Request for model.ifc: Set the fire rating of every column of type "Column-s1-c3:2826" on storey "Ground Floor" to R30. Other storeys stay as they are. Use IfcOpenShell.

First a look at what the model holds.

```python
import ifcopenshell
import ifcopenshell.util.element

model = ifcopenshell.open("model.ifc")
print(model.schema)
storey = next(s for s in model.by_type("IfcBuildingStorey") if s.Name == "Ground Floor")
columns = [e for e in ifcopenshell.util.element.get_decomposition(storey) if e.is_a("IfcColumn")]
seen = {}
for e in columns:
    element_type = ifcopenshell.util.element.get_type(e)
    key = (element_type.Name if element_type != e and element_type else None, ifcopenshell.util.element.get_pset(e, "Pset_ColumnCommon", "FireRating"))
    seen[key] = seen.get(key, 0) + 1
for (name, value), count in sorted(seen.items(), key=str):
    print(count, "x", name, "|", value)
```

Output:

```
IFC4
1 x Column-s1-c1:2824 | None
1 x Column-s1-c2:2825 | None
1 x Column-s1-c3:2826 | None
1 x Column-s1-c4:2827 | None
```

```python
import ifcopenshell
import ifcopenshell.api.pset
import ifcopenshell.util.element

model = ifcopenshell.open("model.ifc")

storey = next(s for s in model.by_type("IfcBuildingStorey") if s.Name == "Ground Floor")
columns = [e for e in ifcopenshell.util.element.get_decomposition(storey) if e.is_a("IfcColumn")]

count = 0
for e in columns:
    element_type = ifcopenshell.util.element.get_type(e)
    if element_type in (None, e) or element_type.Name != "Column-s1-c3:2826":
        continue
    # add_pset returns the element's existing set when there is one.
    pset = ifcopenshell.api.pset.add_pset(model, product=e, name="Pset_ColumnCommon")
    ifcopenshell.api.pset.edit_pset(model, pset=pset, properties={"FireRating": "R30"})
    count += 1

print(count, "columns updated")

model.write("model-out.ifc")
```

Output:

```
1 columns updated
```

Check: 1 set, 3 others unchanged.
